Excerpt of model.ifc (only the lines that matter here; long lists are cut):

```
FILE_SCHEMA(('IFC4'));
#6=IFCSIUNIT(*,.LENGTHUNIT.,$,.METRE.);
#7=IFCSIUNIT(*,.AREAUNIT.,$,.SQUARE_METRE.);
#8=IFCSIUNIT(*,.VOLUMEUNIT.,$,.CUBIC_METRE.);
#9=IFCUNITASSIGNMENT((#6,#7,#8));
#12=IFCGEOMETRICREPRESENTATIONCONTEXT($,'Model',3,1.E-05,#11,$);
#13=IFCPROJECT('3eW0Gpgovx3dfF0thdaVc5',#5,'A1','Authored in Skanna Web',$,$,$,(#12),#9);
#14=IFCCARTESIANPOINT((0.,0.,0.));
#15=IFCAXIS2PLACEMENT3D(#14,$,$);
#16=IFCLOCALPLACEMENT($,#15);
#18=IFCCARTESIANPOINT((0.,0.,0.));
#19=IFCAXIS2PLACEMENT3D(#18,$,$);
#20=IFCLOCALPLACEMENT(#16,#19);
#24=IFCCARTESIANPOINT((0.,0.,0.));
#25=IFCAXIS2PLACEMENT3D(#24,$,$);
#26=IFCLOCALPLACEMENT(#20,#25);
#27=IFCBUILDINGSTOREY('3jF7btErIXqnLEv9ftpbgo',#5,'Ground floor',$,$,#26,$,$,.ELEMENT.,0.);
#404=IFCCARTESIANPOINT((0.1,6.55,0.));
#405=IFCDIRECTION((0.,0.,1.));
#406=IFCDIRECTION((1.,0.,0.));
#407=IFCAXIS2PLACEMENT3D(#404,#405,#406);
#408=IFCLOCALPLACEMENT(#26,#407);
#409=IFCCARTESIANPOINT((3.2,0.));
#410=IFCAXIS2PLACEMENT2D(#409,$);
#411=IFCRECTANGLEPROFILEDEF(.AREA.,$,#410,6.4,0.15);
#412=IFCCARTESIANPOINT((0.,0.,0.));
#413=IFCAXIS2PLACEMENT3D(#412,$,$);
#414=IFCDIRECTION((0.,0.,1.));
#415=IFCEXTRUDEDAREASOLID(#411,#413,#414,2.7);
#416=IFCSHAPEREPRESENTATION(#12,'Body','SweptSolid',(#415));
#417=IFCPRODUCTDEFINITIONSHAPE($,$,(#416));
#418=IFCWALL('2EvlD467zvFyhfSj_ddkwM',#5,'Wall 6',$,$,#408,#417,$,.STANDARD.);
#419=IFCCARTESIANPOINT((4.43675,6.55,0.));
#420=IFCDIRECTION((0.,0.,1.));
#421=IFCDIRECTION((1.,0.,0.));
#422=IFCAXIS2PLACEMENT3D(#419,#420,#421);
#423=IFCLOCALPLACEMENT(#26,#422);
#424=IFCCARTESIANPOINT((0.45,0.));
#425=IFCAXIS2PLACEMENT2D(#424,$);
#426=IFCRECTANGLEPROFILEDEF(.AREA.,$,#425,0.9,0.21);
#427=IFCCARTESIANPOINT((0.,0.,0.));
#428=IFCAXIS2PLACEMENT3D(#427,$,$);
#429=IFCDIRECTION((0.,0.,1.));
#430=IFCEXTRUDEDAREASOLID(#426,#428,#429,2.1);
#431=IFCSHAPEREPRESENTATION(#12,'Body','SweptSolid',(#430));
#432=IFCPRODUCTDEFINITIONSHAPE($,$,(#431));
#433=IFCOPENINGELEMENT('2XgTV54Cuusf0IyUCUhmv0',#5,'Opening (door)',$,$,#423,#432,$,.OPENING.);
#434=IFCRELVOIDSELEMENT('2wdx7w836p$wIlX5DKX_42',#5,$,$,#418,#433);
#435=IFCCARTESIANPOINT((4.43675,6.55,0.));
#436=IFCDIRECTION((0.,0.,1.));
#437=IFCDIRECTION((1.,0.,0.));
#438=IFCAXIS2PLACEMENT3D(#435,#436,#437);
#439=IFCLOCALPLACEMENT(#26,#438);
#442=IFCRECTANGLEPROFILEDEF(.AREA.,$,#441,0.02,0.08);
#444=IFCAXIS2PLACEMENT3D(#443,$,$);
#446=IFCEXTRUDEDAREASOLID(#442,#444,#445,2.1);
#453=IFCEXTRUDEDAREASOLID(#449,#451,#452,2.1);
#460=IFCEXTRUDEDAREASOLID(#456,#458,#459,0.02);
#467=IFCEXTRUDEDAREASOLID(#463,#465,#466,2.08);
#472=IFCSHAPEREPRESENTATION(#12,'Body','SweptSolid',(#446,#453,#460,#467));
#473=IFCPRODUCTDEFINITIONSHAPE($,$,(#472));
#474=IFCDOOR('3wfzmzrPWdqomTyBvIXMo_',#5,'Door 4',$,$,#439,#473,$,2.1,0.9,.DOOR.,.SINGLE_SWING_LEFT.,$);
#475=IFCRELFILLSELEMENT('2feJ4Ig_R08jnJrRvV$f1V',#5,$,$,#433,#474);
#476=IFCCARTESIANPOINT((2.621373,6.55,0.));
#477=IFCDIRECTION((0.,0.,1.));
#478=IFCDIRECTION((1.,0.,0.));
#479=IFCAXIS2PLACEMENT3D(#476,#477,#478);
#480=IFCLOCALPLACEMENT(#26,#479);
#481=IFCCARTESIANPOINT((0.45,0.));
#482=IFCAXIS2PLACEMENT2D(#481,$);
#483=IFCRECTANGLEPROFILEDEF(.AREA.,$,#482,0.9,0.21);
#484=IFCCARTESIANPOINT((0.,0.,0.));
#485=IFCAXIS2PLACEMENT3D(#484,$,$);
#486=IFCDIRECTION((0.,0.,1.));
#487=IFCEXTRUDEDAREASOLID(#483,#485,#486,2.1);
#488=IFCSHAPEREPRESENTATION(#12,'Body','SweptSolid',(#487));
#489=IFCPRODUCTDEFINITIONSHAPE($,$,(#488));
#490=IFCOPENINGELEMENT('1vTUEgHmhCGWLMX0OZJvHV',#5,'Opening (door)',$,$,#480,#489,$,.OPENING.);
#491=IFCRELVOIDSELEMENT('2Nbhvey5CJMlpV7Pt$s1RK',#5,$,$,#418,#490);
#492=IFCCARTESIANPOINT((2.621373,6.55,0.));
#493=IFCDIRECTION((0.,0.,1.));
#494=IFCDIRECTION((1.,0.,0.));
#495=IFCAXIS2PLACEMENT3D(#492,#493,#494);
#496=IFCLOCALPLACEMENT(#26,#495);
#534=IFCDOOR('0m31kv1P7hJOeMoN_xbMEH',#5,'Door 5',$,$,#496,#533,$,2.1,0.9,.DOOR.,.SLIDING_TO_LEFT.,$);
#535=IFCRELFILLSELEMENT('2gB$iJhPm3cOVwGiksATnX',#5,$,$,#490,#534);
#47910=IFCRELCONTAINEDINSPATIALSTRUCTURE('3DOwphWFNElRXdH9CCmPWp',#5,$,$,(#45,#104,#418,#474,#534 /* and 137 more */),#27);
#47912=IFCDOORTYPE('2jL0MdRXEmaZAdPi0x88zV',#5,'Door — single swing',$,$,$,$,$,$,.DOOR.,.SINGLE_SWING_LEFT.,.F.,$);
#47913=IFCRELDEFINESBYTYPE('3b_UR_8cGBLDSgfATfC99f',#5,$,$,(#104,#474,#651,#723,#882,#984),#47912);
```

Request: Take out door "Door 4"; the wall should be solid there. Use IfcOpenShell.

```python
import ifcopenshell
import ifcopenshell.api.feature
import ifcopenshell.api.root
import ifcopenshell.geom
import ifcopenshell.util.shape

model = ifcopenshell.open("model.ifc")
settings = ifcopenshell.geom.settings()


def volume(element):
    """Net volume in cubic metres, openings subtracted."""
    shape = ifcopenshell.geom.create_shape(settings, element)
    return ifcopenshell.util.shape.get_volume(shape.geometry)


door = model.by_guid("3wfzmzrPWdqomTyBvIXMo_")
opening = door.FillsVoids[0].RelatingOpeningElement
wall = opening.VoidsElements[0].RelatingBuildingElement
before = volume(wall)

ifcopenshell.api.root.remove_product(model, product=door)
ifcopenshell.api.feature.remove_feature(model, feature=opening)

after = volume(wall)

print(f"wall volume {before:.3f} -> {after:.3f} m3")

model.write("model-out.ifc")
```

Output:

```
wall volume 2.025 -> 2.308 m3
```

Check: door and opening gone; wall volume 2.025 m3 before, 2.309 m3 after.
